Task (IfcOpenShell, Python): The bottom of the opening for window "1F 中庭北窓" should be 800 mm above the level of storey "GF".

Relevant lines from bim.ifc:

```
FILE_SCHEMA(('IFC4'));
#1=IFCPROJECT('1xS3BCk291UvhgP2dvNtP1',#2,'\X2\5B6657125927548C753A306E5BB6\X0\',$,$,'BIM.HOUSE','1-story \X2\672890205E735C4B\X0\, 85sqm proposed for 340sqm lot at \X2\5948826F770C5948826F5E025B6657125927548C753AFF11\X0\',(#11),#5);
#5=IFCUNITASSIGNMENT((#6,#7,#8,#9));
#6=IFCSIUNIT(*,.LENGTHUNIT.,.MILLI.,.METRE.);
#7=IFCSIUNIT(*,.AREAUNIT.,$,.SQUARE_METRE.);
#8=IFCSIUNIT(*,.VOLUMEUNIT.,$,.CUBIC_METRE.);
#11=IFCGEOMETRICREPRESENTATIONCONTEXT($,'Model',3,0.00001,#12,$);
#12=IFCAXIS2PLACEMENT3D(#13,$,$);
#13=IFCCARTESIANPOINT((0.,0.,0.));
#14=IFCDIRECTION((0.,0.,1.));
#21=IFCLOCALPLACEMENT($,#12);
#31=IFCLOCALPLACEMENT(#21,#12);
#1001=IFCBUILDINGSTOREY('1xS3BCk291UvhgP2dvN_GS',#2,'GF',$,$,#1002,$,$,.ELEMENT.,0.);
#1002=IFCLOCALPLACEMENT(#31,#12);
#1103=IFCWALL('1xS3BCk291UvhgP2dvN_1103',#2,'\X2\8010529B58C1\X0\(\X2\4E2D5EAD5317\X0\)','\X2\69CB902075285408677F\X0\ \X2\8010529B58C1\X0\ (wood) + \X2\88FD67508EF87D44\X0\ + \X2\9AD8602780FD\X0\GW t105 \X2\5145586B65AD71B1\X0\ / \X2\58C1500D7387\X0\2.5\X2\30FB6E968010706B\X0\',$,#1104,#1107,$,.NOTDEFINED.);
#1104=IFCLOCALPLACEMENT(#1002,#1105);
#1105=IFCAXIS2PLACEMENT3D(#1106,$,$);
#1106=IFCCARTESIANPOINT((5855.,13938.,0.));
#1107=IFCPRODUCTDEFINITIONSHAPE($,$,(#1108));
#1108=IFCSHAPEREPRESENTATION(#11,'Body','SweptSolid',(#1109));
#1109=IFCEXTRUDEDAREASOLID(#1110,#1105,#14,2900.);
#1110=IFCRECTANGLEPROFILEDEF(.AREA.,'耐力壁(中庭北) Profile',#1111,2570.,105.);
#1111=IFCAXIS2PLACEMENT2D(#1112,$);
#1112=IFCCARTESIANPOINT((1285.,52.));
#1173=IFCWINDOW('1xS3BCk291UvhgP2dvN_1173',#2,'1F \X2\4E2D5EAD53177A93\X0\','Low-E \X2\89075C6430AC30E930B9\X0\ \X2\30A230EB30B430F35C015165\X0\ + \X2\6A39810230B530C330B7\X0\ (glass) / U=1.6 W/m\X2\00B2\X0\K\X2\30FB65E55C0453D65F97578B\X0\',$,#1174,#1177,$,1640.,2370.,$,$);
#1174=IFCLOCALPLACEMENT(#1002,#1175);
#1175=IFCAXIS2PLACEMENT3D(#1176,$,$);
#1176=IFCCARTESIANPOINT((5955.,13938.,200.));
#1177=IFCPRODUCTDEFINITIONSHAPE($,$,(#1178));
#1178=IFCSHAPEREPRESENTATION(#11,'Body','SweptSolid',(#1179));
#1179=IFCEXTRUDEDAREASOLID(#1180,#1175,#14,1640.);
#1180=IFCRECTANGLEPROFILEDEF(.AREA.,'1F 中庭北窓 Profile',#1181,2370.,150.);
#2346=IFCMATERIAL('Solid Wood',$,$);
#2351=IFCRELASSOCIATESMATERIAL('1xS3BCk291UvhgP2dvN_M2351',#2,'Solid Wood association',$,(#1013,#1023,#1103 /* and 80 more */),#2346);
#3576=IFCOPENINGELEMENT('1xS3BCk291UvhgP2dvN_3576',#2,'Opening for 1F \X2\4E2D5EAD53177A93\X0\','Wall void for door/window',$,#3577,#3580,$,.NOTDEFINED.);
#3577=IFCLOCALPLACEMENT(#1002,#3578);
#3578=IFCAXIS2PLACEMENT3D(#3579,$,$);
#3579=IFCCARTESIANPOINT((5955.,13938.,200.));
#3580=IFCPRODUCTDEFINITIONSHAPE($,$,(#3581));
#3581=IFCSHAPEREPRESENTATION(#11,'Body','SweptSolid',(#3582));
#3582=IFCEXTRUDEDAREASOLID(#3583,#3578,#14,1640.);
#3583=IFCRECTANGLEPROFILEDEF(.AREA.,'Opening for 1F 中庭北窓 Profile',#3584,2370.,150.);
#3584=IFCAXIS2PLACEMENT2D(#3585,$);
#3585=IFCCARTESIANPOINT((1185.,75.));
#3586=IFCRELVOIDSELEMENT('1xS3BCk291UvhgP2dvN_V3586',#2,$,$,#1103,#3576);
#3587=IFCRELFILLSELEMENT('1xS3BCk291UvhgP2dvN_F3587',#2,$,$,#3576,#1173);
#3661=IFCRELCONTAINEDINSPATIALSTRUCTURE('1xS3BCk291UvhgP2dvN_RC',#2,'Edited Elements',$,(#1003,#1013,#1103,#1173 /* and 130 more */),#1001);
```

```python
import numpy as np
import ifcopenshell
import ifcopenshell.api.geometry
import ifcopenshell.geom
import ifcopenshell.util.element
import ifcopenshell.util.placement
import ifcopenshell.util.shape
import ifcopenshell.util.unit

model = ifcopenshell.open("bim.ifc")
unit_scale = ifcopenshell.util.unit.calculate_unit_scale(model)

window = model.by_guid("1xS3BCk291UvhgP2dvN_1173")
opening = window.FillsVoids[0].RelatingOpeningElement
storey = ifcopenshell.util.element.get_container(window, ifc_class="IfcBuildingStorey")
level = ifcopenshell.util.placement.get_local_placement(storey.ObjectPlacement)[2, 3]

# The opening's origin need not be at the sill, so measure its lowest point.
shape = ifcopenshell.geom.create_shape(ifcopenshell.geom.settings(), opening)
bottom = ifcopenshell.util.shape.get_shape_bottom_elevation(shape, shape.geometry) / unit_scale
dz = level + 0.8 / unit_scale - bottom

shift = np.array([0.0, 0.0, dz])
# The window is not placed relative to its opening, so move both.
for product in (opening, window):
    matrix = ifcopenshell.util.placement.get_local_placement(product.ObjectPlacement)
    matrix[:3, 3] += shift
    ifcopenshell.api.geometry.edit_object_placement(model, product=product, matrix=matrix, is_si=False)

print(f"moved by {dz * unit_scale:+.3f} m")

model.write("bim-out.ifc")
```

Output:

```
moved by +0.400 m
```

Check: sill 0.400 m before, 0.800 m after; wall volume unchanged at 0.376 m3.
